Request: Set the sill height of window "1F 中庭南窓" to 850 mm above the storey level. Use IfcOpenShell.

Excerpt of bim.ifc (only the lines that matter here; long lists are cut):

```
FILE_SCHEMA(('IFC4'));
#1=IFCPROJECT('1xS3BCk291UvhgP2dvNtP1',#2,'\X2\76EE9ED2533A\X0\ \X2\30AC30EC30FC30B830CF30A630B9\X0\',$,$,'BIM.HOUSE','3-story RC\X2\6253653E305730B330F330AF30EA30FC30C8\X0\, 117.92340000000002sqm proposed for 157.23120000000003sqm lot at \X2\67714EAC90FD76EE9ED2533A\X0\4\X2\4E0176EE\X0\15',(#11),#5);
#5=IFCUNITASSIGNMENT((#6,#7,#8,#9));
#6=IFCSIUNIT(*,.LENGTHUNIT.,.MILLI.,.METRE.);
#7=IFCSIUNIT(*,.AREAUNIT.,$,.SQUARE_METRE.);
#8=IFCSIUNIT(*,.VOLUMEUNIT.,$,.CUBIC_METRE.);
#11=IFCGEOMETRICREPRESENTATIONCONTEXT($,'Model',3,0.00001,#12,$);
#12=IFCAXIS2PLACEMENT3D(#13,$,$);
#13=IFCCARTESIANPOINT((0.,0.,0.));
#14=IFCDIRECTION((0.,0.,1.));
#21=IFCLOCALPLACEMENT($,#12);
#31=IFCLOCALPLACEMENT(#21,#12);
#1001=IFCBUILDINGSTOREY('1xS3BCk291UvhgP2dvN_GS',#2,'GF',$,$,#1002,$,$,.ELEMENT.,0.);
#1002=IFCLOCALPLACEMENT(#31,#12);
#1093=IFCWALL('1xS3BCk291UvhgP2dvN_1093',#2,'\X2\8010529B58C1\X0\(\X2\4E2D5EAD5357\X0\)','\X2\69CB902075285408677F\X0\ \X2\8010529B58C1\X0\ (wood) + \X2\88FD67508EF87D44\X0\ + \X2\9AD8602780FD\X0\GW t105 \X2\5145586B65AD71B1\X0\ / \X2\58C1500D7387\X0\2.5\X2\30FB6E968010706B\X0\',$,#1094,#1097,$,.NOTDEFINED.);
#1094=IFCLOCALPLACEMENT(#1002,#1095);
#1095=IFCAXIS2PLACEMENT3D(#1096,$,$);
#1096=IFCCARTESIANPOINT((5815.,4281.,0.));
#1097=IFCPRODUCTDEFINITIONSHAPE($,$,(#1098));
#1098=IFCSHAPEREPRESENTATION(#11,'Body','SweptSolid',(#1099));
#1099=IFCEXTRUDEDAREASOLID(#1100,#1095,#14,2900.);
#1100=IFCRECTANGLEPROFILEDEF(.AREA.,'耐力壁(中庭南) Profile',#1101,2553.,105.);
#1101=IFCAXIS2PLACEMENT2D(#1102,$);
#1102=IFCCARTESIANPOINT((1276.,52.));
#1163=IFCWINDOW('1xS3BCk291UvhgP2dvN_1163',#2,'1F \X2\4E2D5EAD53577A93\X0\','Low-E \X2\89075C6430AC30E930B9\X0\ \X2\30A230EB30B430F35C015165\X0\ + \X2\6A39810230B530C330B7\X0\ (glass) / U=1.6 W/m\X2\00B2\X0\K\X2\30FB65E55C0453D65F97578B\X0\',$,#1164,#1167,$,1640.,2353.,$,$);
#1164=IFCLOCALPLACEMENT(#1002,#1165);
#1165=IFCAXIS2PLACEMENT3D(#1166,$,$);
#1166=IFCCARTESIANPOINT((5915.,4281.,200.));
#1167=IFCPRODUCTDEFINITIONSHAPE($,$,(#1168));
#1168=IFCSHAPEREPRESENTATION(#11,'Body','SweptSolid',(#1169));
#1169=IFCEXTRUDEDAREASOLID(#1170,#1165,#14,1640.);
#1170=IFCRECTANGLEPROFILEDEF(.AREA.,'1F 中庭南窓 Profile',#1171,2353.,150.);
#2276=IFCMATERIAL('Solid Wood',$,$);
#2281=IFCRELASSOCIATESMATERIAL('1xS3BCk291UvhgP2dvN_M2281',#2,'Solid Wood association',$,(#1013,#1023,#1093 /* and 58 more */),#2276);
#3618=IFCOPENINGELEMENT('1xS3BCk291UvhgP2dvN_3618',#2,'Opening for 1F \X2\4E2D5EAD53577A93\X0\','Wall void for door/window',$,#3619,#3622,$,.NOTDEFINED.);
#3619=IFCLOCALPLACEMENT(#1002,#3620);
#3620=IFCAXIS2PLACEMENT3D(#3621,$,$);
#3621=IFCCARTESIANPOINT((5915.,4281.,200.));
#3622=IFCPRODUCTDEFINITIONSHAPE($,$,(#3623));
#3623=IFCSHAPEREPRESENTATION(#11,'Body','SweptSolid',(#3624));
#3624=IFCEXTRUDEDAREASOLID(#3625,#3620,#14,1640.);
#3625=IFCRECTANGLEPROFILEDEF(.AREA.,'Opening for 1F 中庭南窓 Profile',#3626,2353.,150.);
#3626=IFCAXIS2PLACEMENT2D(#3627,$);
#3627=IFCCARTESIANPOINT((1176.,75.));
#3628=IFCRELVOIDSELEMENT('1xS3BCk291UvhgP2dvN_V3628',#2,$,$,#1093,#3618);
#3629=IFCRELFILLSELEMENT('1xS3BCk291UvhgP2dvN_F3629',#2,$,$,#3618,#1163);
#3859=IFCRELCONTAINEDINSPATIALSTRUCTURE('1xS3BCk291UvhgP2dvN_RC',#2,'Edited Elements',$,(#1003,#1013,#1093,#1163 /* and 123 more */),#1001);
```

```python
import numpy as np
import ifcopenshell
import ifcopenshell.api.geometry
import ifcopenshell.geom
import ifcopenshell.util.element
import ifcopenshell.util.placement
import ifcopenshell.util.shape
import ifcopenshell.util.unit

model = ifcopenshell.open("bim.ifc")
unit_scale = ifcopenshell.util.unit.calculate_unit_scale(model)

window = model.by_guid("1xS3BCk291UvhgP2dvN_1163")
opening = window.FillsVoids[0].RelatingOpeningElement
storey = ifcopenshell.util.element.get_container(window, ifc_class="IfcBuildingStorey")
level = ifcopenshell.util.placement.get_local_placement(storey.ObjectPlacement)[2, 3]

# The opening's origin need not be at the sill, so measure its lowest point.
shape = ifcopenshell.geom.create_shape(ifcopenshell.geom.settings(), opening)
bottom = ifcopenshell.util.shape.get_shape_bottom_elevation(shape, shape.geometry) / unit_scale
dz = level + 0.85 / unit_scale - bottom

shift = np.array([0.0, 0.0, dz])
# The window is not placed relative to its opening, so move both.
for product in (opening, window):
    matrix = ifcopenshell.util.placement.get_local_placement(product.ObjectPlacement)
    matrix[:3, 3] += shift
    ifcopenshell.api.geometry.edit_object_placement(model, product=product, matrix=matrix, is_si=False)

print(f"moved by {dz * unit_scale:+.3f} m")

model.write("bim_updated.ifc")
```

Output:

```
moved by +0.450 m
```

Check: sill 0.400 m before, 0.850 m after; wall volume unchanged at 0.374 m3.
